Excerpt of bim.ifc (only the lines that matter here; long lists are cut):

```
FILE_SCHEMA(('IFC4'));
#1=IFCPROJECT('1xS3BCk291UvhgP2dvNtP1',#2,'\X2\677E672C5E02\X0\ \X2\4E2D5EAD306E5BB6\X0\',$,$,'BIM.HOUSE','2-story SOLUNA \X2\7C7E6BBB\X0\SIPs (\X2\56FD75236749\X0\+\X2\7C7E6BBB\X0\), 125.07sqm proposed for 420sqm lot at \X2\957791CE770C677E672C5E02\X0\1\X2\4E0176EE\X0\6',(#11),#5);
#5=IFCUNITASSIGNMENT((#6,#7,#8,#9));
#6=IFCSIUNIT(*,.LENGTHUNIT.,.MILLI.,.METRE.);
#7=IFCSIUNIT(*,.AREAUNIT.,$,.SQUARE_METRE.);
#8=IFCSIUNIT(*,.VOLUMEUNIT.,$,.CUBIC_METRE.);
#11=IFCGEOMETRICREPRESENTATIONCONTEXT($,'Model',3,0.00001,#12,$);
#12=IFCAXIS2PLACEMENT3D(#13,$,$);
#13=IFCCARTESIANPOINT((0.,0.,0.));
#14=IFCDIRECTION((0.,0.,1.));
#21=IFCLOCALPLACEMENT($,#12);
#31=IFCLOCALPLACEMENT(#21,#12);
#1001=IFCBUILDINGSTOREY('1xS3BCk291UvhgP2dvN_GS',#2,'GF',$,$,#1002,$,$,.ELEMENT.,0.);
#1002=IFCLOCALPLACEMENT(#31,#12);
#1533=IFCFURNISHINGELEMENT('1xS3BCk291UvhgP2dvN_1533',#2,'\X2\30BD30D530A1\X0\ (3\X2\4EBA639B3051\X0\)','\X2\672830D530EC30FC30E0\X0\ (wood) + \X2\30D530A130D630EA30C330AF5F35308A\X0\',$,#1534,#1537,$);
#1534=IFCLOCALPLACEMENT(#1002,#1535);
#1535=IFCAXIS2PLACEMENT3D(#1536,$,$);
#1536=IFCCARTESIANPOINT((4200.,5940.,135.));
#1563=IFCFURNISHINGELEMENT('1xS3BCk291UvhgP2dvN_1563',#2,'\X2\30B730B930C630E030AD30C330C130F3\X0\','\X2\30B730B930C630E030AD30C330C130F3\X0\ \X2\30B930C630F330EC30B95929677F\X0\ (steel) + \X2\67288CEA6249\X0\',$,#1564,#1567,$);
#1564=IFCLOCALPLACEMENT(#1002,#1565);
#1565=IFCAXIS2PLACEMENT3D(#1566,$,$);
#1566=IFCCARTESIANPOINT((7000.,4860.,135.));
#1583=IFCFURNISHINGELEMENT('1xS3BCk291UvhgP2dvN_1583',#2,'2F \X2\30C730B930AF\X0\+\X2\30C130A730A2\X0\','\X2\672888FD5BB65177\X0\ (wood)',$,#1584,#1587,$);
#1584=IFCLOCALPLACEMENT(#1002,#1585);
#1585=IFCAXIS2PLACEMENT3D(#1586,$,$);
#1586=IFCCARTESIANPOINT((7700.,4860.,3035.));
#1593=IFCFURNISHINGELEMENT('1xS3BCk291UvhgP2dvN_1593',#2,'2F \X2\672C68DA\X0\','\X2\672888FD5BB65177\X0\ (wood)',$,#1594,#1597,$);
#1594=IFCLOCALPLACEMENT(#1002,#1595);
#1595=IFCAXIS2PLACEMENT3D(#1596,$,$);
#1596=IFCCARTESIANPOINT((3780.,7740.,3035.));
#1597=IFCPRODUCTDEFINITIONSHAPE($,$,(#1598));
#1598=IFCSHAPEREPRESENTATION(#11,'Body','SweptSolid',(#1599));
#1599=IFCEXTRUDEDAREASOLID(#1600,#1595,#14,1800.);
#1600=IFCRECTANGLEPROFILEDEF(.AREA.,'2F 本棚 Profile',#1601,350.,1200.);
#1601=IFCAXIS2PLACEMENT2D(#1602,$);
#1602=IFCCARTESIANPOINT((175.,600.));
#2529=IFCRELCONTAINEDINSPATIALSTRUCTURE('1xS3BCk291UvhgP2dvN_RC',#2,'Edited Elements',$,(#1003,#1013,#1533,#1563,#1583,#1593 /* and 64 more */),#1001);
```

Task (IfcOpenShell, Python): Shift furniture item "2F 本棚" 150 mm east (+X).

```python
import ifcopenshell
import ifcopenshell.api.geometry
import ifcopenshell.util.placement
import ifcopenshell.util.unit

model = ifcopenshell.open("bim.ifc")
unit_scale = ifcopenshell.util.unit.calculate_unit_scale(model)

item = model.by_id(1593)
matrix = ifcopenshell.util.placement.get_local_placement(item.ObjectPlacement)
matrix[0, 3] += 0.15 / unit_scale
ifcopenshell.api.geometry.edit_object_placement(model, product=item, matrix=matrix, is_si=False)

print(ifcopenshell.util.placement.get_local_placement(item.ObjectPlacement).round(3) + 0.0)

model.write("bim-out.ifc")
```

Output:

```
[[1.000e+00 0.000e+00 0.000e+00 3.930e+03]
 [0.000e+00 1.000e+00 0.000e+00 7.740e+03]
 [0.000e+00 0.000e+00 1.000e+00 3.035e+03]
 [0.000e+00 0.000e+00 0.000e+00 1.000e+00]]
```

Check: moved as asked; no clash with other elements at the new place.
